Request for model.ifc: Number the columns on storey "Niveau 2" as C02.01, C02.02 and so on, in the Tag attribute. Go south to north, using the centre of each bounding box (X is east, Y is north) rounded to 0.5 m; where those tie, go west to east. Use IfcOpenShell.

First a look at what the model holds.

```python
import ifcopenshell
import ifcopenshell.util.element
import ifcopenshell.util.placement

model = ifcopenshell.open("model.ifc")
print(model.schema)
storey = next(s for s in model.by_type("IfcBuildingStorey") if s.Name == "Niveau 2")
columns = [e for e in ifcopenshell.util.element.get_decomposition(storey) if e.is_a("IfcColumn")]
for e in sorted(columns, key=lambda e: e.id()):
    origin = ifcopenshell.util.placement.get_local_placement(e.ObjectPlacement)[:3, 3]
    print(e.id(), e.Tag, e.Name, origin.round(2) + 0.0, sep=" | ")
```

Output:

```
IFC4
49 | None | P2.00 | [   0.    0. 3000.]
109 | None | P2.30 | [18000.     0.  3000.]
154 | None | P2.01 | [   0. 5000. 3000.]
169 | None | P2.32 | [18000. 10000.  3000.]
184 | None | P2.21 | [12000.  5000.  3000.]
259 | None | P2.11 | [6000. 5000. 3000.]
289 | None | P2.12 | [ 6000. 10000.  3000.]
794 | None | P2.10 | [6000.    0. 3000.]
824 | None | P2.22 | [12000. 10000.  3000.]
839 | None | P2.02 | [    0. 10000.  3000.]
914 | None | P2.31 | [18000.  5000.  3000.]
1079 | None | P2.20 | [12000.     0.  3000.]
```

```python
import ifcopenshell
import ifcopenshell.geom
import ifcopenshell.util.element
import ifcopenshell.util.shape

model = ifcopenshell.open("model.ifc")
settings = ifcopenshell.geom.settings()
settings.set("use-world-coords", True)


def centre(element):
    shape = ifcopenshell.geom.create_shape(settings, element)
    return ifcopenshell.util.shape.get_bbox_centroid(shape.geometry)


storey = next(s for s in model.by_type("IfcBuildingStorey") if s.Name == "Niveau 2")
columns = [e for e in ifcopenshell.util.element.get_decomposition(storey) if e.is_a("IfcColumn")]

# Insertion points can sit at a corner or the storey origin, so sort by the geometry (in metres).
centres = {e: centre(e) for e in columns}
columns.sort(key=lambda e: (round(centres[e][1] / 0.5), centres[e][0]))

for i, e in enumerate(columns, start=1):
    number = f"C02.{i:02d}"
    e.Tag = number
    print(e.id(), number)

model.write("model-out.ifc")
```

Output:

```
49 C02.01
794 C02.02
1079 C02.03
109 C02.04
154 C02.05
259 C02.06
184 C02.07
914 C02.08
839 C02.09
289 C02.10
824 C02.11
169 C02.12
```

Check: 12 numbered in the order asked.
